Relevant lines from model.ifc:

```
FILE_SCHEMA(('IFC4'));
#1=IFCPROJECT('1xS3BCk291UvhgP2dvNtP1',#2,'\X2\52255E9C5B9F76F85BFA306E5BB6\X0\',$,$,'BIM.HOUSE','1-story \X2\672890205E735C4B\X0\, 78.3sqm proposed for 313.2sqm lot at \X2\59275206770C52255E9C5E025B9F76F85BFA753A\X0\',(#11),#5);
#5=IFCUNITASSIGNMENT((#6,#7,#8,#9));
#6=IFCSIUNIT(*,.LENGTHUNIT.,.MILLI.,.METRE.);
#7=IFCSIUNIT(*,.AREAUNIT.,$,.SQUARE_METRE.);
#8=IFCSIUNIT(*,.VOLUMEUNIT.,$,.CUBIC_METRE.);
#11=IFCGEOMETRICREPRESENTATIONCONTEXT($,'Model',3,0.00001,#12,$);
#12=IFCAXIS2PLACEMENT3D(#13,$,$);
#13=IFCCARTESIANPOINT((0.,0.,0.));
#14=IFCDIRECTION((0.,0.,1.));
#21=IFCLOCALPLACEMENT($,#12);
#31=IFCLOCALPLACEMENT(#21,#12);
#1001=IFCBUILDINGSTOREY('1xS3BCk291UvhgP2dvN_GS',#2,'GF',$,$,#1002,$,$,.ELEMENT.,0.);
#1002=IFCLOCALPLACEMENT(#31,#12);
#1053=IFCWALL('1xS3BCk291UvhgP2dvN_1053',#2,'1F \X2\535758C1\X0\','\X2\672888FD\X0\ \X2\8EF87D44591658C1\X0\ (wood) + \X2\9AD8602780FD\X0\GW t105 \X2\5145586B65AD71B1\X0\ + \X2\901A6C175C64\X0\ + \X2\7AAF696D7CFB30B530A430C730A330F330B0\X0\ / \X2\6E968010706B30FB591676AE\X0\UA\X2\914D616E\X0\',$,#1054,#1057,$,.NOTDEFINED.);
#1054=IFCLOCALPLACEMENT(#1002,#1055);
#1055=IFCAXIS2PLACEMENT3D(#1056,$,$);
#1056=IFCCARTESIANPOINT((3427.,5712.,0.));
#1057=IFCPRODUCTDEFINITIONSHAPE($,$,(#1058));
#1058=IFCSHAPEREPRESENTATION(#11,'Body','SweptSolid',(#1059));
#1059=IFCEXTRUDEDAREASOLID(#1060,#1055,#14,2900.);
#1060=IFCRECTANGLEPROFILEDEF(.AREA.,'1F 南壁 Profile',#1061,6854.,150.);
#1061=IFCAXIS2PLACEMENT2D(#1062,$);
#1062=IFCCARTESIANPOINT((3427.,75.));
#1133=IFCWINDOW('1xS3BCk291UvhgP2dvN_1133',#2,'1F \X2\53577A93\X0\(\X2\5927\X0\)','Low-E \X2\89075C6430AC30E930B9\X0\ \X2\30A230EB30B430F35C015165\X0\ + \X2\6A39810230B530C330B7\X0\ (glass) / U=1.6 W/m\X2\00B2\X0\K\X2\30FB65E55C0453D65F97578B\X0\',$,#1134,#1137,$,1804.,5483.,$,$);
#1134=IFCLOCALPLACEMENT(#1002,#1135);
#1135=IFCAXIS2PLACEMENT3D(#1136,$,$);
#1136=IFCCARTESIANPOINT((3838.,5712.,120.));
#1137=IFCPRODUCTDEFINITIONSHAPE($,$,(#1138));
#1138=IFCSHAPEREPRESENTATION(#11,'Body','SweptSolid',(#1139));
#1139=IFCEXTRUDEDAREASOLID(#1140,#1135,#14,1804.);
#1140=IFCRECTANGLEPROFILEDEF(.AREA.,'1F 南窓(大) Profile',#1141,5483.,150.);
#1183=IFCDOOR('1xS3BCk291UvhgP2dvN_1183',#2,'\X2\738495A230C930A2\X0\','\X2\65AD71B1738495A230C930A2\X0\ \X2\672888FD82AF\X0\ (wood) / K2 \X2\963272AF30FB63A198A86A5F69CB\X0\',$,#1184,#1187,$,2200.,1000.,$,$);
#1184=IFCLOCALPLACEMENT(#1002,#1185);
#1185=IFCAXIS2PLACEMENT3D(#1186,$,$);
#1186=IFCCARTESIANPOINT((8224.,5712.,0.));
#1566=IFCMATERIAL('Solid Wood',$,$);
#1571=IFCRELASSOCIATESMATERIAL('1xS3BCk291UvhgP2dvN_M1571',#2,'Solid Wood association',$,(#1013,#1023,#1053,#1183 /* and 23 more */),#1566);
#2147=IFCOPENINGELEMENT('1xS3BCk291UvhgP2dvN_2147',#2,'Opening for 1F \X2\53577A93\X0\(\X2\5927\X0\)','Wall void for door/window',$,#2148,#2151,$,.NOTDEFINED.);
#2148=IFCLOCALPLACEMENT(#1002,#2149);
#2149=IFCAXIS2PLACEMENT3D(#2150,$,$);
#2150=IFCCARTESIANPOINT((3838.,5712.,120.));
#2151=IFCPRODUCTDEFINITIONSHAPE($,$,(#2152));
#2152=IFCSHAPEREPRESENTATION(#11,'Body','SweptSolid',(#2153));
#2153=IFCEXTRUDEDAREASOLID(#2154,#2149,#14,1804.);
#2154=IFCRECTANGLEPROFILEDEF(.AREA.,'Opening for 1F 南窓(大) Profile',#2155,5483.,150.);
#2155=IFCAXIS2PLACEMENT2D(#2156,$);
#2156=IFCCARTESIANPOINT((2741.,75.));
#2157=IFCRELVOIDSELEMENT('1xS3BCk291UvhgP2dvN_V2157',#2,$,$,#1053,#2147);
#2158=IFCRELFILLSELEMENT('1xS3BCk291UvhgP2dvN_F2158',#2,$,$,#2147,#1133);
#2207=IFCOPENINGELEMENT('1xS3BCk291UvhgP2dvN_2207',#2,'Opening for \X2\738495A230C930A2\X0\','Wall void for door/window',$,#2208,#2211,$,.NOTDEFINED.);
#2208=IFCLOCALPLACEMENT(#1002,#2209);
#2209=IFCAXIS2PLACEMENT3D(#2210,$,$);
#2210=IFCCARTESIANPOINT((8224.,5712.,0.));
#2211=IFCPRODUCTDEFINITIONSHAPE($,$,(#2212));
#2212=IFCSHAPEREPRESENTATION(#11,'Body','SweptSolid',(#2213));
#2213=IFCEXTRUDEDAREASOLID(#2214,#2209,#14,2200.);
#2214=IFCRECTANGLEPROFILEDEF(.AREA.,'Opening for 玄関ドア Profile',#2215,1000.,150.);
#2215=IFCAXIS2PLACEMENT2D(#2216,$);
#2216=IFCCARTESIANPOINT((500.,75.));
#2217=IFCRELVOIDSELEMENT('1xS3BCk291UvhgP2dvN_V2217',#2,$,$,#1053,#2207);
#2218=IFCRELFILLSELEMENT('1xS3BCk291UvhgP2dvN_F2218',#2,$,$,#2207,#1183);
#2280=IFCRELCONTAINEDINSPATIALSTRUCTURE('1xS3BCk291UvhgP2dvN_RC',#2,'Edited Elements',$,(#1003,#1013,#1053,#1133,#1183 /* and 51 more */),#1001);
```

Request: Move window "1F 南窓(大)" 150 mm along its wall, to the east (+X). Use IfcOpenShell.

```python
import ifcopenshell
import ifcopenshell.api.geometry
import ifcopenshell.util.placement

model = ifcopenshell.open("model.ifc")

window = model.by_guid("1xS3BCk291UvhgP2dvN_1133")
opening = window.FillsVoids[0].RelatingOpeningElement
wall = opening.VoidsElements[0].RelatingBuildingElement

wall_matrix = ifcopenshell.util.placement.get_local_placement(wall.ObjectPlacement)
shift = wall_matrix[:3, 0] * 150.0
before = ifcopenshell.util.placement.get_local_placement(window.ObjectPlacement)[:3, 3].copy()

# The window is not placed relative to its opening, so move both.
for product in (opening, window):
    matrix = ifcopenshell.util.placement.get_local_placement(product.ObjectPlacement)
    matrix[:3, 3] += shift
    ifcopenshell.api.geometry.edit_object_placement(model, product=product, matrix=matrix, is_si=False)

after = ifcopenshell.util.placement.get_local_placement(window.ObjectPlacement)[:3, 3]
print("window moved by", (after - before).round(3) + 0.0)

model.write("model_rev.ifc")
```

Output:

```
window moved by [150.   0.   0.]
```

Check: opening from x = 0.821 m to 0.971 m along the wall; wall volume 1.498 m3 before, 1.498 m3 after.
